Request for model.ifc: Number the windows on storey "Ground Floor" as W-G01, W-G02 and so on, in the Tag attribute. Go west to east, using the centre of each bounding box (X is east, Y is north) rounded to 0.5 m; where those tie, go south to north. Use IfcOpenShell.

First a look at what the model holds.

```python
import ifcopenshell
import ifcopenshell.util.element
import ifcopenshell.util.placement

model = ifcopenshell.open("model.ifc")
print(model.schema)
storey = next(s for s in model.by_type("IfcBuildingStorey") if s.Name == "Ground Floor")
windows = [e for e in ifcopenshell.util.element.get_decomposition(storey) if e.is_a("IfcWindow")]
for e in sorted(windows, key=lambda e: e.id()):
    origin = ifcopenshell.util.placement.get_local_placement(e.ObjectPlacement)[:3, 3]
    print(e.id(), e.Tag, e.Name, origin.round(2) + 0.0, sep=" | ")
```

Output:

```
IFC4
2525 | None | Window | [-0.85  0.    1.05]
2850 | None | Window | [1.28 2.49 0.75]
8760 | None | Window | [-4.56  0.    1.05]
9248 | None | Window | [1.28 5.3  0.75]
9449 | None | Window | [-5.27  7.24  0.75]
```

```python
import ifcopenshell
import ifcopenshell.geom
import ifcopenshell.util.element
import ifcopenshell.util.shape

model = ifcopenshell.open("model.ifc")
settings = ifcopenshell.geom.settings()
settings.set("use-world-coords", True)


def centre(element):
    shape = ifcopenshell.geom.create_shape(settings, element)
    return ifcopenshell.util.shape.get_bbox_centroid(shape.geometry)


storey = next(s for s in model.by_type("IfcBuildingStorey") if s.Name == "Ground Floor")
windows = [e for e in ifcopenshell.util.element.get_decomposition(storey) if e.is_a("IfcWindow")]

# Insertion points can sit at a corner or the storey origin, so sort by the geometry (in metres).
centres = {e: centre(e) for e in windows}
windows.sort(key=lambda e: (round(centres[e][0] / 0.5), centres[e][1]))

for i, e in enumerate(windows, start=1):
    number = f"W-G{i:02d}"
    e.Tag = number
    print(e.id(), number)

model.write("model_rev.ifc")
```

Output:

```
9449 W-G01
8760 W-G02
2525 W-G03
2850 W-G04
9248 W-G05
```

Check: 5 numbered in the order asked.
